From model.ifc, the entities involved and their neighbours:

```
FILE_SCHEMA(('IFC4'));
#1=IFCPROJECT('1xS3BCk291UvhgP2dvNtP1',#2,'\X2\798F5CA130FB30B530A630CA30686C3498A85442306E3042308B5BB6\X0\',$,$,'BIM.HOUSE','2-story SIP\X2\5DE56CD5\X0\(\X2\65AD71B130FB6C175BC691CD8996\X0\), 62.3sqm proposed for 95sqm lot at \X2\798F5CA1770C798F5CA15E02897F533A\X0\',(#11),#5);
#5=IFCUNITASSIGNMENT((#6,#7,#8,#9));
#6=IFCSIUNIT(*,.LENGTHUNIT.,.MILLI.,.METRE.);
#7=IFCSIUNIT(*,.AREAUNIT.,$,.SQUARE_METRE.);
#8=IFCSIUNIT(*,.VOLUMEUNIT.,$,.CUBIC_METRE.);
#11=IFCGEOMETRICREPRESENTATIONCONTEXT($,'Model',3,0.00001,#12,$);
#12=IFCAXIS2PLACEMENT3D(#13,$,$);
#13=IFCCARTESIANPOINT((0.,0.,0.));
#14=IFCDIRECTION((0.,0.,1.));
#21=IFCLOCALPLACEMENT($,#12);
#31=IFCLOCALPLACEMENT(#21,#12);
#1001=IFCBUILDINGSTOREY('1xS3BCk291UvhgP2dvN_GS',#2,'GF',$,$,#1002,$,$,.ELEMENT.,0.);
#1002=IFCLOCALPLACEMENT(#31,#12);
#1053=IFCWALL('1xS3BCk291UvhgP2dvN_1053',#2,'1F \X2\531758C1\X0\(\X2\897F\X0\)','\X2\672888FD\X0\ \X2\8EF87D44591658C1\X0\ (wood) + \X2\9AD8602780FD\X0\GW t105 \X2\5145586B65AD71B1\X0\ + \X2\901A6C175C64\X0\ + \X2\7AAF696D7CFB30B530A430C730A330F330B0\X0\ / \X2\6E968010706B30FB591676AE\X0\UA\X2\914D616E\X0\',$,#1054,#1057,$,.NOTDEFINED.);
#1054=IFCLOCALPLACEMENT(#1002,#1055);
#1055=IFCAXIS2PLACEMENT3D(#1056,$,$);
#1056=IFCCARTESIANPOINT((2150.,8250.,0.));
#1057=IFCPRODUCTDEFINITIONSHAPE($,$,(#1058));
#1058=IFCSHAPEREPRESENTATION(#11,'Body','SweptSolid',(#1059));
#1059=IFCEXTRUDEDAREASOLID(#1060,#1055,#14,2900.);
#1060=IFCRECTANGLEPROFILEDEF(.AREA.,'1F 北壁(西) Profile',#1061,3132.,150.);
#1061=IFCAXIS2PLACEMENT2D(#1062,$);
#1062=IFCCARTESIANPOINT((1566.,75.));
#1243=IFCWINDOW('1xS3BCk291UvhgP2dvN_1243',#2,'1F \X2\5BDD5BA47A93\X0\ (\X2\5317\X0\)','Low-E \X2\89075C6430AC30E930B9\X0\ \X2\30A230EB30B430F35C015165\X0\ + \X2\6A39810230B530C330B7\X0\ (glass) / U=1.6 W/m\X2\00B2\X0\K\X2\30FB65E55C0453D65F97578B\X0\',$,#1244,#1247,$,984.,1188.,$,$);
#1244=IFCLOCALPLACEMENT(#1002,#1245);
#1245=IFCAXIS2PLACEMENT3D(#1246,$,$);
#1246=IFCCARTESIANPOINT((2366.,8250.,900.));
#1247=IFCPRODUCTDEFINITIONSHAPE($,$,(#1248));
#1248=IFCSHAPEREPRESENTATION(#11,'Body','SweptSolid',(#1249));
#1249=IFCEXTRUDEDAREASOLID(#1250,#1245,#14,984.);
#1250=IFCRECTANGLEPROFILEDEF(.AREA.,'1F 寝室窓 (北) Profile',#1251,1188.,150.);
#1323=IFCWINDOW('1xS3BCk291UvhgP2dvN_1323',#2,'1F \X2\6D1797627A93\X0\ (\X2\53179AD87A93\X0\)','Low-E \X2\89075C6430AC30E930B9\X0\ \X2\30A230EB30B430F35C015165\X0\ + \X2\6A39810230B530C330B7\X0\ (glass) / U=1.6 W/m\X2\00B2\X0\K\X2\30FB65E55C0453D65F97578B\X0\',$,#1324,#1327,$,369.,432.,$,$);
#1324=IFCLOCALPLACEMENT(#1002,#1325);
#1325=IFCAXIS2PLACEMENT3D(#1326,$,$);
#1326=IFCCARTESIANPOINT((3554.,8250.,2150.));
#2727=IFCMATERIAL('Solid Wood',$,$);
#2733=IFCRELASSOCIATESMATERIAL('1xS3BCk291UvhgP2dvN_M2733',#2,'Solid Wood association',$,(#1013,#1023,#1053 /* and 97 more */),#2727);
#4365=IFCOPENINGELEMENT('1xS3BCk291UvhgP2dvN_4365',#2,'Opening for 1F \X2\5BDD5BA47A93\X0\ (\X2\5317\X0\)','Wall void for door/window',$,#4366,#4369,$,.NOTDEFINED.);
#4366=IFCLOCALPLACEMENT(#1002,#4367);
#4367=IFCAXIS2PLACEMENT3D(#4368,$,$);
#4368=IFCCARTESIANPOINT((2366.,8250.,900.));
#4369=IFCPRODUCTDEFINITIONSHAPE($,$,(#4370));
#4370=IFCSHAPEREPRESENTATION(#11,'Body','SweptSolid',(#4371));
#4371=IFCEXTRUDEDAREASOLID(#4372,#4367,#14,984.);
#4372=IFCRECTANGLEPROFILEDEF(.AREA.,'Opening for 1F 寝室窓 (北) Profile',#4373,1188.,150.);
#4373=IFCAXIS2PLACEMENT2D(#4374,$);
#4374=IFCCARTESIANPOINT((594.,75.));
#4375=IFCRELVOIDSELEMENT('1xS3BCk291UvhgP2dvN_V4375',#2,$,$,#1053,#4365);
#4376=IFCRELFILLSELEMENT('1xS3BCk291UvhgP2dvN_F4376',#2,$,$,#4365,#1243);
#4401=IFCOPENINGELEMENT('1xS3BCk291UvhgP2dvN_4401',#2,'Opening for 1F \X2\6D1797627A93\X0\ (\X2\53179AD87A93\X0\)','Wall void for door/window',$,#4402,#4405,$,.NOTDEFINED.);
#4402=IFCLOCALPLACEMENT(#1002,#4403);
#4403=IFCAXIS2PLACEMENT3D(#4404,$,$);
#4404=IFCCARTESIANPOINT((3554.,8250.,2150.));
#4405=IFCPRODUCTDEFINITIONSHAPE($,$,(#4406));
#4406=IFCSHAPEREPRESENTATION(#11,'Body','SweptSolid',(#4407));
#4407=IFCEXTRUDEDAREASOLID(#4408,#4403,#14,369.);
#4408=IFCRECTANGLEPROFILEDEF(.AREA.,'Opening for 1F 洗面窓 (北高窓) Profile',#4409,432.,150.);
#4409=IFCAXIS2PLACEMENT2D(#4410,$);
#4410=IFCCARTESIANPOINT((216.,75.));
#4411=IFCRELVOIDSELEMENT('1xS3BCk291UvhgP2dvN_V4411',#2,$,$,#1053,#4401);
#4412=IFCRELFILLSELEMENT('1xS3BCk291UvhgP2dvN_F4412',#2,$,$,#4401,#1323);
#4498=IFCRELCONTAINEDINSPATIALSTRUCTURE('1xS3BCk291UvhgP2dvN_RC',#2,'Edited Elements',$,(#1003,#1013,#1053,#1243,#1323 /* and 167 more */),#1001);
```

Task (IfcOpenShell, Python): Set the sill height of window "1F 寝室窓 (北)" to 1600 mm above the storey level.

```python
import numpy as np
import ifcopenshell
import ifcopenshell.api.geometry
import ifcopenshell.geom
import ifcopenshell.util.element
import ifcopenshell.util.placement
import ifcopenshell.util.shape
import ifcopenshell.util.unit

model = ifcopenshell.open("model.ifc")
unit_scale = ifcopenshell.util.unit.calculate_unit_scale(model)

window = model.by_guid("1xS3BCk291UvhgP2dvN_1243")
opening = window.FillsVoids[0].RelatingOpeningElement
storey = ifcopenshell.util.element.get_container(window, ifc_class="IfcBuildingStorey")
level = ifcopenshell.util.placement.get_local_placement(storey.ObjectPlacement)[2, 3]

# The opening's origin need not be at the sill, so measure its lowest point.
shape = ifcopenshell.geom.create_shape(ifcopenshell.geom.settings(), opening)
bottom = ifcopenshell.util.shape.get_shape_bottom_elevation(shape, shape.geometry) / unit_scale
dz = level + 1600.0 - bottom

shift = np.array([0.0, 0.0, dz])
# The window is not placed relative to its opening, so move both.
for product in (opening, window):
    matrix = ifcopenshell.util.placement.get_local_placement(product.ObjectPlacement)
    matrix[:3, 3] += shift
    ifcopenshell.api.geometry.edit_object_placement(model, product=product, matrix=matrix, is_si=False)

print(f"moved by {dz * unit_scale:+.3f} m")

model.write("model-out.ifc")
```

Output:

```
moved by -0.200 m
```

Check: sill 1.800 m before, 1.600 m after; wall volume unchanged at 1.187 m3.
